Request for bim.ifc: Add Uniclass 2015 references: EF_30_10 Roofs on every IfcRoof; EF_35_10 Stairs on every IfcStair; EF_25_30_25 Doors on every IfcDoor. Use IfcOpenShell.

First a look at what the model holds.

```python
import ifcopenshell

model = ifcopenshell.open("bim.ifc")
print(model.schema)
print("classifications:", [c.Name for c in model.by_type("IfcClassification")])
for ifc_class in ("IfcDoor", "IfcRoof", "IfcStair", "IfcWall", "IfcWindow"):
    print(ifc_class, len(model.by_type(ifc_class)))
```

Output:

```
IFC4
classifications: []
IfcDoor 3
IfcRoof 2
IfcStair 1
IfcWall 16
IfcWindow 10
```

```python
import ifcopenshell
import ifcopenshell.api.classification

model = ifcopenshell.open("bim.ifc")

system = ifcopenshell.api.classification.add_classification(model, classification="Uniclass 2015")

codes = {
    "IfcRoof": ("EF_30_10", "Roofs"),
    "IfcStair": ("EF_35_10", "Stairs"),
    "IfcDoor": ("EF_25_30_25", "Doors"),
}
for ifc_class, (code, name) in codes.items():
    products = model.by_type(ifc_class)
    ifcopenshell.api.classification.add_reference(
        model, products=products, classification=system, identification=code, name=name
    )
    print(code, len(products))

model.write("bim_v2.ifc")
```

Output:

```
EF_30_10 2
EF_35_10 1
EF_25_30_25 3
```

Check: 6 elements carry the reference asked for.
